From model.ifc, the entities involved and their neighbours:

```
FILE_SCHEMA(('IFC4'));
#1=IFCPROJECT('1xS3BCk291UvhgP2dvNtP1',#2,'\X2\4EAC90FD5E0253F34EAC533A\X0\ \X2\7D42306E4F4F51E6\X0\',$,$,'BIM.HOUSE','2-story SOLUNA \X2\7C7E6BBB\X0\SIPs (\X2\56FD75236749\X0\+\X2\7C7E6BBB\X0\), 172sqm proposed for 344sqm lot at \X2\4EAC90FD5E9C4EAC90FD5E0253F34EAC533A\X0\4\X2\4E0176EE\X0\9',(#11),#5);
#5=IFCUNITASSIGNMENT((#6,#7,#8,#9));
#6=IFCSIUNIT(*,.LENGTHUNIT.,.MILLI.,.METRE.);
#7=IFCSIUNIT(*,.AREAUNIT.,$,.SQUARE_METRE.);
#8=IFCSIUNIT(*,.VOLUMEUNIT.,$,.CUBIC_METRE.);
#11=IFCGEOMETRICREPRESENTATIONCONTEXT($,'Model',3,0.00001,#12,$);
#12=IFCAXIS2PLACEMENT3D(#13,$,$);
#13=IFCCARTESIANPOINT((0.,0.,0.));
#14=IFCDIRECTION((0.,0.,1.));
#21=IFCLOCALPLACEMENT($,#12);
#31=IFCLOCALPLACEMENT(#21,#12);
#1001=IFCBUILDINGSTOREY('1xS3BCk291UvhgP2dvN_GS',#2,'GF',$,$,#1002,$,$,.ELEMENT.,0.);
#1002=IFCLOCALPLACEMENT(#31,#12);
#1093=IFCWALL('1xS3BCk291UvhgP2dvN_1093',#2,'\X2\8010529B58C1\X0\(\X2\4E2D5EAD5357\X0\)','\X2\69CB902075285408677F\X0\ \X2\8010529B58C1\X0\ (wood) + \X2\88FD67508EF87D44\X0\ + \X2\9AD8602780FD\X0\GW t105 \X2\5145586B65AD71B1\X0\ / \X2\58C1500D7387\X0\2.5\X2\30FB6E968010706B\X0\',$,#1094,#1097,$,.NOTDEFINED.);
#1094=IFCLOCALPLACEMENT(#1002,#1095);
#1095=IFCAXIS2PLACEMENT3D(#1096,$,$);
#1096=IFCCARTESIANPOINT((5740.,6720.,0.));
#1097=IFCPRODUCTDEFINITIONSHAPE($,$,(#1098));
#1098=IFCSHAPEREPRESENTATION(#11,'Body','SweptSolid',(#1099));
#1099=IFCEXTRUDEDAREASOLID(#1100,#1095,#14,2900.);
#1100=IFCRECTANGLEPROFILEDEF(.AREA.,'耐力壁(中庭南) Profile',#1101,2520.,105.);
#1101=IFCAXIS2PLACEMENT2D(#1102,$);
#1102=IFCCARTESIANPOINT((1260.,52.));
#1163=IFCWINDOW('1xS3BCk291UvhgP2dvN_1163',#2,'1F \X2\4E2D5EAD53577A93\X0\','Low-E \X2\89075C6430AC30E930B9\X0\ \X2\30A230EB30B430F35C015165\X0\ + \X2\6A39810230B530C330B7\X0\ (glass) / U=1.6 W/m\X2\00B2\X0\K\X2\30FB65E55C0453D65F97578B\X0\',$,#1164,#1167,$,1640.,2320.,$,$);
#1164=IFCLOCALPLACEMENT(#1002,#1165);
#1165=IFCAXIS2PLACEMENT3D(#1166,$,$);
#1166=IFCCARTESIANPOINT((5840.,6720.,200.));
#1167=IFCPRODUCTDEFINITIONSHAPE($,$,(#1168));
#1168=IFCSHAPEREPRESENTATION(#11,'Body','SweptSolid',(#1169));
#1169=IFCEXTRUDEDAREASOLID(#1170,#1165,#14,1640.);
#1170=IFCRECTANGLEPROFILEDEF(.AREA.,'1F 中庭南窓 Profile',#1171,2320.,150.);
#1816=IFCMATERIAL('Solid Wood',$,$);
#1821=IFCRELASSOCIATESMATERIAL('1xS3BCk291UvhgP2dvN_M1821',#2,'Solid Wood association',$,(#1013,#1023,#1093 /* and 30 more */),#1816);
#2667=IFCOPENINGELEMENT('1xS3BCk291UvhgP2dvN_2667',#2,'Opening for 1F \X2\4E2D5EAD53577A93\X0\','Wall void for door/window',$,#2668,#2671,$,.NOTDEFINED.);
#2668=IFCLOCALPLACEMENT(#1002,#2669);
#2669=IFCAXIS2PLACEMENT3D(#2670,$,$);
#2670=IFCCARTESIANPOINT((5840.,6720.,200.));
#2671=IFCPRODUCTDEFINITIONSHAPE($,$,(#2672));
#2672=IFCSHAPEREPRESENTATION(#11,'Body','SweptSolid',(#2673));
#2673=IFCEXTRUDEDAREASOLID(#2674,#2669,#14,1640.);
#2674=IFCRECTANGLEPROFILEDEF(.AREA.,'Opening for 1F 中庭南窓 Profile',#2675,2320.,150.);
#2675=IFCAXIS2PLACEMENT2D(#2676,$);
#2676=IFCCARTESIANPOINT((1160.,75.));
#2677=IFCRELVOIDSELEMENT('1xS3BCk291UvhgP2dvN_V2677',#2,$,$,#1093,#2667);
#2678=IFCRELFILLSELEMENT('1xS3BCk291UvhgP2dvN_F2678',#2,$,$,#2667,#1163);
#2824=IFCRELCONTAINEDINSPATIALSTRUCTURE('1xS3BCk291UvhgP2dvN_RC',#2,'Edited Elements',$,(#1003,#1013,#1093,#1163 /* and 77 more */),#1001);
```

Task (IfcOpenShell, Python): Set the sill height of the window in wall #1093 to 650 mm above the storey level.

```python
import numpy as np
import ifcopenshell
import ifcopenshell.api.geometry
import ifcopenshell.geom
import ifcopenshell.util.element
import ifcopenshell.util.placement
import ifcopenshell.util.shape
import ifcopenshell.util.unit

model = ifcopenshell.open("model.ifc")
unit_scale = ifcopenshell.util.unit.calculate_unit_scale(model)

window = model.by_guid("1xS3BCk291UvhgP2dvN_1163")
opening = window.FillsVoids[0].RelatingOpeningElement
storey = ifcopenshell.util.element.get_container(window, ifc_class="IfcBuildingStorey")
level = ifcopenshell.util.placement.get_local_placement(storey.ObjectPlacement)[2, 3]

# The opening's origin need not be at the sill, so measure its lowest point.
shape = ifcopenshell.geom.create_shape(ifcopenshell.geom.settings(), opening)
bottom = ifcopenshell.util.shape.get_shape_bottom_elevation(shape, shape.geometry) / unit_scale
dz = level + 0.65 / unit_scale - bottom

shift = np.array([0.0, 0.0, dz])
# The window is not placed relative to its opening, so move both.
for product in (opening, window):
    matrix = ifcopenshell.util.placement.get_local_placement(product.ObjectPlacement)
    matrix[:3, 3] += shift
    ifcopenshell.api.geometry.edit_object_placement(model, product=product, matrix=matrix, is_si=False)

print(f"moved by {dz * unit_scale:+.3f} m")

model.write("model_v2.ifc")
```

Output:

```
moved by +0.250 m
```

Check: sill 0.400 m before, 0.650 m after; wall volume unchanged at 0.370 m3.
